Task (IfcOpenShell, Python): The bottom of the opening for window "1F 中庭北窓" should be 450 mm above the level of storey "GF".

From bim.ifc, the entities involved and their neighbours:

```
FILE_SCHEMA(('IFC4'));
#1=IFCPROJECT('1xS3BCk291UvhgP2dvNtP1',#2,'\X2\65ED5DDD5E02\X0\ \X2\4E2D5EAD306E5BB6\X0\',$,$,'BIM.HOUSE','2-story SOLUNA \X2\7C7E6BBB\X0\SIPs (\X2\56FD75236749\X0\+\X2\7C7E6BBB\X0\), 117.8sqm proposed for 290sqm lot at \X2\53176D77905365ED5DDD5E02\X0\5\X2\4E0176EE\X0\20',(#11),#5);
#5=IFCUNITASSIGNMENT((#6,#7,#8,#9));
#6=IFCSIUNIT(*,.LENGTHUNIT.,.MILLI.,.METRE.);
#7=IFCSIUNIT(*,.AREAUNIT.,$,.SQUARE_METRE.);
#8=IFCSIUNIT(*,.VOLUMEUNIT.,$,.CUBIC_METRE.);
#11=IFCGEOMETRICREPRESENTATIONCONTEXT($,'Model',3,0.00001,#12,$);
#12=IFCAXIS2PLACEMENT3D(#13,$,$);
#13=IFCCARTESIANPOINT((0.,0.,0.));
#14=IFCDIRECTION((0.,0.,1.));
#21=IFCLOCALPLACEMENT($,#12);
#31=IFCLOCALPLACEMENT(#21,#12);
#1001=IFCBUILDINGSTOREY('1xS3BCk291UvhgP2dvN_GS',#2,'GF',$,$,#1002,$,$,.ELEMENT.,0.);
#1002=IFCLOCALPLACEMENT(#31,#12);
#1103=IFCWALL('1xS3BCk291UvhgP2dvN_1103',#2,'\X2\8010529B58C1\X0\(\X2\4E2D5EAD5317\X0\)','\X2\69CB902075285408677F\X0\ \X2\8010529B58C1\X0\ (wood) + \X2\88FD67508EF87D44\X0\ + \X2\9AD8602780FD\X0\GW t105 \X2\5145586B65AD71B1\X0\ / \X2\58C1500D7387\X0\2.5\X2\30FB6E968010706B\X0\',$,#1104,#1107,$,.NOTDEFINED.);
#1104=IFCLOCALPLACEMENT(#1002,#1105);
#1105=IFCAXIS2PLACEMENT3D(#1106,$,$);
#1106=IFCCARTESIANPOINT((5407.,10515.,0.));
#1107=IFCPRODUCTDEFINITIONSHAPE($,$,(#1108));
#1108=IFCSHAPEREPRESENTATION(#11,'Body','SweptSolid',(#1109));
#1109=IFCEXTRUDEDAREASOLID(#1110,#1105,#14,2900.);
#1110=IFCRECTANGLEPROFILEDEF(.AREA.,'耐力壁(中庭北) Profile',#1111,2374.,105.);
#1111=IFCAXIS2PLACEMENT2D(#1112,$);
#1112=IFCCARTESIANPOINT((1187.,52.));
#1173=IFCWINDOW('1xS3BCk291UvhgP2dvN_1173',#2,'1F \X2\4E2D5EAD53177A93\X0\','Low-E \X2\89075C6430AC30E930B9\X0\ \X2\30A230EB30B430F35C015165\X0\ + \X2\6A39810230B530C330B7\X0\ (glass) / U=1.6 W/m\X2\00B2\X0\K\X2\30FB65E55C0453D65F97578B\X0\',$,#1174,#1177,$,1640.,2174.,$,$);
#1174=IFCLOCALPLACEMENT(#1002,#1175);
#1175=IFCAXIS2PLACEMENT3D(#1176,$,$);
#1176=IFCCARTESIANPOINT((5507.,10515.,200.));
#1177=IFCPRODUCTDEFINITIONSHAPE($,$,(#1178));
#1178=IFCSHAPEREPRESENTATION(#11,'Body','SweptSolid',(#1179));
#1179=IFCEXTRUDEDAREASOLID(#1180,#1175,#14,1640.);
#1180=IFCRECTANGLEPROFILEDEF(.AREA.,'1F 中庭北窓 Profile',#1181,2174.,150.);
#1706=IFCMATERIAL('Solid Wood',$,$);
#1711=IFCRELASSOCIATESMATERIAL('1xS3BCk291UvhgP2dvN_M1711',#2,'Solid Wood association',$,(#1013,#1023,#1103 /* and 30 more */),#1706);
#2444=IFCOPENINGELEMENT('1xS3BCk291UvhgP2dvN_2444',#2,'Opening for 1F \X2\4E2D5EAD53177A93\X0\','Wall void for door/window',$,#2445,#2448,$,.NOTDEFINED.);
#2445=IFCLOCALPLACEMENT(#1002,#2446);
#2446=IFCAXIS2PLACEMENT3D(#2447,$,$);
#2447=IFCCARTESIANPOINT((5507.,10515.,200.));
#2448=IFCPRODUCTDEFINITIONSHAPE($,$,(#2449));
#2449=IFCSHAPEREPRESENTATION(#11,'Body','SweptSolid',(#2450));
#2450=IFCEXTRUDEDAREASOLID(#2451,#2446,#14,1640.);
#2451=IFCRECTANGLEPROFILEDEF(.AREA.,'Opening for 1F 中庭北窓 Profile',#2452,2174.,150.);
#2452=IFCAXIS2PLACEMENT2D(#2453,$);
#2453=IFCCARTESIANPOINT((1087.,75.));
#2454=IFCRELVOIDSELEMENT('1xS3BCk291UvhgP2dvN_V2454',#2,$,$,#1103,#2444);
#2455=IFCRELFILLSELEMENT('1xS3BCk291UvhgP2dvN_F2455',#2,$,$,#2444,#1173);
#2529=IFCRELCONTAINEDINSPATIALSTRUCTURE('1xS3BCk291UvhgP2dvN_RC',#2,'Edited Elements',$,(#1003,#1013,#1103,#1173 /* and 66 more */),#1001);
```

```python
import numpy as np
import ifcopenshell
import ifcopenshell.api.geometry
import ifcopenshell.geom
import ifcopenshell.util.element
import ifcopenshell.util.placement
import ifcopenshell.util.shape
import ifcopenshell.util.unit

model = ifcopenshell.open("bim.ifc")
unit_scale = ifcopenshell.util.unit.calculate_unit_scale(model)

window = model.by_id(1173)
opening = window.FillsVoids[0].RelatingOpeningElement
storey = ifcopenshell.util.element.get_container(window, ifc_class="IfcBuildingStorey")
level = ifcopenshell.util.placement.get_local_placement(storey.ObjectPlacement)[2, 3]

# The opening's origin need not be at the sill, so measure its lowest point.
shape = ifcopenshell.geom.create_shape(ifcopenshell.geom.settings(), opening)
bottom = ifcopenshell.util.shape.get_shape_bottom_elevation(shape, shape.geometry) / unit_scale
dz = level + 0.45 / unit_scale - bottom

shift = np.array([0.0, 0.0, dz])
# The window is not placed relative to its opening, so move both.
for product in (opening, window):
    matrix = ifcopenshell.util.placement.get_local_placement(product.ObjectPlacement)
    matrix[:3, 3] += shift
    ifcopenshell.api.geometry.edit_object_placement(model, product=product, matrix=matrix, is_si=False)

print(f"moved by {dz * unit_scale:+.3f} m")

model.write("bim_updated.ifc")
```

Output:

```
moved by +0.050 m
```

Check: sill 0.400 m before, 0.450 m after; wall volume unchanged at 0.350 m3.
